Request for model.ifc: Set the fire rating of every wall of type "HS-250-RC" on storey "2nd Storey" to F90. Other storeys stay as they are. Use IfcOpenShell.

First a look at what the model holds.

```python
import ifcopenshell
import ifcopenshell.util.element

model = ifcopenshell.open("model.ifc")
print(model.schema)
storey = next(s for s in model.by_type("IfcBuildingStorey") if s.Name == "2nd Storey")
walls = [e for e in ifcopenshell.util.element.get_decomposition(storey) if e.is_a("IfcWall")]
seen = {}
for e in walls:
    element_type = ifcopenshell.util.element.get_type(e)
    key = (element_type.Name if element_type != e and element_type else None, ifcopenshell.util.element.get_pset(e, "Pset_WallCommon", "FireRating"))
    seen[key] = seen.get(key, 0) + 1
for (name, value), count in sorted(seen.items(), key=str):
    print(count, "x", name, "|", value)
```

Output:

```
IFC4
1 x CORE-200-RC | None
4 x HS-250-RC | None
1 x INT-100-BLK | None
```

```python
import ifcopenshell
import ifcopenshell.api.pset
import ifcopenshell.util.element

model = ifcopenshell.open("model.ifc")

storey = next(s for s in model.by_type("IfcBuildingStorey") if s.Name == "2nd Storey")
walls = [e for e in ifcopenshell.util.element.get_decomposition(storey) if e.is_a("IfcWall")]

count = 0
for e in walls:
    element_type = ifcopenshell.util.element.get_type(e)
    if element_type in (None, e) or element_type.Name != "HS-250-RC":
        continue
    # add_pset returns the element's existing set when there is one.
    pset = ifcopenshell.api.pset.add_pset(model, product=e, name="Pset_WallCommon")
    ifcopenshell.api.pset.edit_pset(model, pset=pset, properties={"FireRating": "F90"})
    count += 1

print(count, "walls updated")

model.write("model-out.ifc")
```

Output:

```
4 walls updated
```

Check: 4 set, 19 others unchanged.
